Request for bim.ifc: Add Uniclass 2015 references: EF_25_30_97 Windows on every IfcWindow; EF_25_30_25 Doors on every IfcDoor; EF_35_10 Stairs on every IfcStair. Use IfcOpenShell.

First a look at what the model holds.

```python
import ifcopenshell

model = ifcopenshell.open("bim.ifc")
print(model.schema)
print("classifications:", [c.Name for c in model.by_type("IfcClassification")])
for ifc_class in ("IfcDoor", "IfcRoof", "IfcStair", "IfcWall", "IfcWindow"):
    print(ifc_class, len(model.by_type(ifc_class)))
```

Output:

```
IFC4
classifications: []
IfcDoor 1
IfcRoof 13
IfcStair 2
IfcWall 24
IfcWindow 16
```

```python
import ifcopenshell
import ifcopenshell.api.classification

model = ifcopenshell.open("bim.ifc")

system = ifcopenshell.api.classification.add_classification(model, classification="Uniclass 2015")

codes = {
    "IfcWindow": ("EF_25_30_97", "Windows"),
    "IfcDoor": ("EF_25_30_25", "Doors"),
    "IfcStair": ("EF_35_10", "Stairs"),
}
for ifc_class, (code, name) in codes.items():
    products = model.by_type(ifc_class)
    ifcopenshell.api.classification.add_reference(
        model, products=products, classification=system, identification=code, name=name
    )
    print(code, len(products))

model.write("bim_rev.ifc")
```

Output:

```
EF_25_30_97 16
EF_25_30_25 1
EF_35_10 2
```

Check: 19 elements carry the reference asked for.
